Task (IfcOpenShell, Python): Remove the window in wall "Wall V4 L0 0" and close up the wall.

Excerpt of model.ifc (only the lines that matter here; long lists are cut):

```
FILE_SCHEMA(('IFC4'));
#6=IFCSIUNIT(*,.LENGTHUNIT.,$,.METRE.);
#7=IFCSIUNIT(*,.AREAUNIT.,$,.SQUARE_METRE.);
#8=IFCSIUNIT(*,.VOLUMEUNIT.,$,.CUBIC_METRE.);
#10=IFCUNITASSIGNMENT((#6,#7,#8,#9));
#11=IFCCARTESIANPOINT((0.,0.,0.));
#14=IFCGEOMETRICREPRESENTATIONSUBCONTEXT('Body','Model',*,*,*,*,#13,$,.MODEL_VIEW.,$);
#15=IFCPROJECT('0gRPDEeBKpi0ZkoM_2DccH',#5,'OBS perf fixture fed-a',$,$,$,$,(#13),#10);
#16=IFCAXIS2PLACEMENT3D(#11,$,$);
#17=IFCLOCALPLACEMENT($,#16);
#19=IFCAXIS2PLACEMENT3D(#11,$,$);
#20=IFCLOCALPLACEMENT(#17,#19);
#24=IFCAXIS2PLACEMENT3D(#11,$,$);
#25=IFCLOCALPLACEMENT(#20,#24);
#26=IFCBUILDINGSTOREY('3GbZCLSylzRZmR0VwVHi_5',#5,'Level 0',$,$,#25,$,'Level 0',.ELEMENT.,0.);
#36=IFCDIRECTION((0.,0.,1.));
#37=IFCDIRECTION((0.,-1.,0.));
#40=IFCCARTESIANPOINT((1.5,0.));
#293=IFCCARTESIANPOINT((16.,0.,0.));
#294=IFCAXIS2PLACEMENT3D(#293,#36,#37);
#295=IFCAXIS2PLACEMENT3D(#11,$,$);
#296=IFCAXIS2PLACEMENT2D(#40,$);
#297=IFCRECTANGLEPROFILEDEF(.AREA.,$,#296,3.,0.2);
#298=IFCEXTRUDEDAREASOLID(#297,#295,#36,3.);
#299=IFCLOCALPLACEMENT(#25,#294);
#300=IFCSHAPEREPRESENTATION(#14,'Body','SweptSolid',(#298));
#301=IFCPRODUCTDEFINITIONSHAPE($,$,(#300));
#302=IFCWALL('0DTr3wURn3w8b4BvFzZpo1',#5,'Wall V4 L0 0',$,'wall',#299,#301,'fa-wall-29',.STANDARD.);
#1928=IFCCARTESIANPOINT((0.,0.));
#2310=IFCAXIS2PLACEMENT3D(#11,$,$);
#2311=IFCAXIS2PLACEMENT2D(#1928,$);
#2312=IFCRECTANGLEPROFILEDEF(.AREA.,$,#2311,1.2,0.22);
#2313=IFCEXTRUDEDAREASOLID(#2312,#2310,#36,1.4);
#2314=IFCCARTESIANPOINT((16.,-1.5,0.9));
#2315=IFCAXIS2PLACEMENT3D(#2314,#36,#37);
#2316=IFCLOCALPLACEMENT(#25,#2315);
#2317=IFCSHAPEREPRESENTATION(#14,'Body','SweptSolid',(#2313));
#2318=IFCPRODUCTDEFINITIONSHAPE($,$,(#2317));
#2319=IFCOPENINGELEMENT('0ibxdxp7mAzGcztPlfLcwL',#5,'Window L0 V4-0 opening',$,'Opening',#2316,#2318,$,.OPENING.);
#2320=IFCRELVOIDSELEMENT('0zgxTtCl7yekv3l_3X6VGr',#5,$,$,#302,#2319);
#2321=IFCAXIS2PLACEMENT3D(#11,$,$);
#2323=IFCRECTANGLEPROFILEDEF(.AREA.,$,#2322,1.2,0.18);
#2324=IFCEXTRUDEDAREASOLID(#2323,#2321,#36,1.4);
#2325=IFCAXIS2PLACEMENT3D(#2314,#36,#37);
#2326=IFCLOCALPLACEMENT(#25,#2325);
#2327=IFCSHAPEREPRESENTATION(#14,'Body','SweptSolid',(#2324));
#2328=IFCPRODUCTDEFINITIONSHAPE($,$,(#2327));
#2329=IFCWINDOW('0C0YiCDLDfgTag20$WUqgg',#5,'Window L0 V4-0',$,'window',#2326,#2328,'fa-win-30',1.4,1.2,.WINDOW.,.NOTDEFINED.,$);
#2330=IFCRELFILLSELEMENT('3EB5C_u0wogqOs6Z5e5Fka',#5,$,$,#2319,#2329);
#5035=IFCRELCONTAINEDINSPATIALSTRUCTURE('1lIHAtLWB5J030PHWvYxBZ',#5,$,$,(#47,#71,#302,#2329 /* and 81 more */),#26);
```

```python
import ifcopenshell
import ifcopenshell.api.feature
import ifcopenshell.api.root
import ifcopenshell.geom
import ifcopenshell.util.shape

model = ifcopenshell.open("model.ifc")
settings = ifcopenshell.geom.settings()


def volume(element):
    """Net volume in cubic metres, openings subtracted."""
    shape = ifcopenshell.geom.create_shape(settings, element)
    return ifcopenshell.util.shape.get_volume(shape.geometry)


window = model.by_id(2329)
opening = window.FillsVoids[0].RelatingOpeningElement
wall = opening.VoidsElements[0].RelatingBuildingElement
before = volume(wall)

ifcopenshell.api.root.remove_product(model, product=window)
ifcopenshell.api.feature.remove_feature(model, feature=opening)

after = volume(wall)

print(f"wall volume {before:.3f} -> {after:.3f} m3")

model.write("model_edited.ifc")
```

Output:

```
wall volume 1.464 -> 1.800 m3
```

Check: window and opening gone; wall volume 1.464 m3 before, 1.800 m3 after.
